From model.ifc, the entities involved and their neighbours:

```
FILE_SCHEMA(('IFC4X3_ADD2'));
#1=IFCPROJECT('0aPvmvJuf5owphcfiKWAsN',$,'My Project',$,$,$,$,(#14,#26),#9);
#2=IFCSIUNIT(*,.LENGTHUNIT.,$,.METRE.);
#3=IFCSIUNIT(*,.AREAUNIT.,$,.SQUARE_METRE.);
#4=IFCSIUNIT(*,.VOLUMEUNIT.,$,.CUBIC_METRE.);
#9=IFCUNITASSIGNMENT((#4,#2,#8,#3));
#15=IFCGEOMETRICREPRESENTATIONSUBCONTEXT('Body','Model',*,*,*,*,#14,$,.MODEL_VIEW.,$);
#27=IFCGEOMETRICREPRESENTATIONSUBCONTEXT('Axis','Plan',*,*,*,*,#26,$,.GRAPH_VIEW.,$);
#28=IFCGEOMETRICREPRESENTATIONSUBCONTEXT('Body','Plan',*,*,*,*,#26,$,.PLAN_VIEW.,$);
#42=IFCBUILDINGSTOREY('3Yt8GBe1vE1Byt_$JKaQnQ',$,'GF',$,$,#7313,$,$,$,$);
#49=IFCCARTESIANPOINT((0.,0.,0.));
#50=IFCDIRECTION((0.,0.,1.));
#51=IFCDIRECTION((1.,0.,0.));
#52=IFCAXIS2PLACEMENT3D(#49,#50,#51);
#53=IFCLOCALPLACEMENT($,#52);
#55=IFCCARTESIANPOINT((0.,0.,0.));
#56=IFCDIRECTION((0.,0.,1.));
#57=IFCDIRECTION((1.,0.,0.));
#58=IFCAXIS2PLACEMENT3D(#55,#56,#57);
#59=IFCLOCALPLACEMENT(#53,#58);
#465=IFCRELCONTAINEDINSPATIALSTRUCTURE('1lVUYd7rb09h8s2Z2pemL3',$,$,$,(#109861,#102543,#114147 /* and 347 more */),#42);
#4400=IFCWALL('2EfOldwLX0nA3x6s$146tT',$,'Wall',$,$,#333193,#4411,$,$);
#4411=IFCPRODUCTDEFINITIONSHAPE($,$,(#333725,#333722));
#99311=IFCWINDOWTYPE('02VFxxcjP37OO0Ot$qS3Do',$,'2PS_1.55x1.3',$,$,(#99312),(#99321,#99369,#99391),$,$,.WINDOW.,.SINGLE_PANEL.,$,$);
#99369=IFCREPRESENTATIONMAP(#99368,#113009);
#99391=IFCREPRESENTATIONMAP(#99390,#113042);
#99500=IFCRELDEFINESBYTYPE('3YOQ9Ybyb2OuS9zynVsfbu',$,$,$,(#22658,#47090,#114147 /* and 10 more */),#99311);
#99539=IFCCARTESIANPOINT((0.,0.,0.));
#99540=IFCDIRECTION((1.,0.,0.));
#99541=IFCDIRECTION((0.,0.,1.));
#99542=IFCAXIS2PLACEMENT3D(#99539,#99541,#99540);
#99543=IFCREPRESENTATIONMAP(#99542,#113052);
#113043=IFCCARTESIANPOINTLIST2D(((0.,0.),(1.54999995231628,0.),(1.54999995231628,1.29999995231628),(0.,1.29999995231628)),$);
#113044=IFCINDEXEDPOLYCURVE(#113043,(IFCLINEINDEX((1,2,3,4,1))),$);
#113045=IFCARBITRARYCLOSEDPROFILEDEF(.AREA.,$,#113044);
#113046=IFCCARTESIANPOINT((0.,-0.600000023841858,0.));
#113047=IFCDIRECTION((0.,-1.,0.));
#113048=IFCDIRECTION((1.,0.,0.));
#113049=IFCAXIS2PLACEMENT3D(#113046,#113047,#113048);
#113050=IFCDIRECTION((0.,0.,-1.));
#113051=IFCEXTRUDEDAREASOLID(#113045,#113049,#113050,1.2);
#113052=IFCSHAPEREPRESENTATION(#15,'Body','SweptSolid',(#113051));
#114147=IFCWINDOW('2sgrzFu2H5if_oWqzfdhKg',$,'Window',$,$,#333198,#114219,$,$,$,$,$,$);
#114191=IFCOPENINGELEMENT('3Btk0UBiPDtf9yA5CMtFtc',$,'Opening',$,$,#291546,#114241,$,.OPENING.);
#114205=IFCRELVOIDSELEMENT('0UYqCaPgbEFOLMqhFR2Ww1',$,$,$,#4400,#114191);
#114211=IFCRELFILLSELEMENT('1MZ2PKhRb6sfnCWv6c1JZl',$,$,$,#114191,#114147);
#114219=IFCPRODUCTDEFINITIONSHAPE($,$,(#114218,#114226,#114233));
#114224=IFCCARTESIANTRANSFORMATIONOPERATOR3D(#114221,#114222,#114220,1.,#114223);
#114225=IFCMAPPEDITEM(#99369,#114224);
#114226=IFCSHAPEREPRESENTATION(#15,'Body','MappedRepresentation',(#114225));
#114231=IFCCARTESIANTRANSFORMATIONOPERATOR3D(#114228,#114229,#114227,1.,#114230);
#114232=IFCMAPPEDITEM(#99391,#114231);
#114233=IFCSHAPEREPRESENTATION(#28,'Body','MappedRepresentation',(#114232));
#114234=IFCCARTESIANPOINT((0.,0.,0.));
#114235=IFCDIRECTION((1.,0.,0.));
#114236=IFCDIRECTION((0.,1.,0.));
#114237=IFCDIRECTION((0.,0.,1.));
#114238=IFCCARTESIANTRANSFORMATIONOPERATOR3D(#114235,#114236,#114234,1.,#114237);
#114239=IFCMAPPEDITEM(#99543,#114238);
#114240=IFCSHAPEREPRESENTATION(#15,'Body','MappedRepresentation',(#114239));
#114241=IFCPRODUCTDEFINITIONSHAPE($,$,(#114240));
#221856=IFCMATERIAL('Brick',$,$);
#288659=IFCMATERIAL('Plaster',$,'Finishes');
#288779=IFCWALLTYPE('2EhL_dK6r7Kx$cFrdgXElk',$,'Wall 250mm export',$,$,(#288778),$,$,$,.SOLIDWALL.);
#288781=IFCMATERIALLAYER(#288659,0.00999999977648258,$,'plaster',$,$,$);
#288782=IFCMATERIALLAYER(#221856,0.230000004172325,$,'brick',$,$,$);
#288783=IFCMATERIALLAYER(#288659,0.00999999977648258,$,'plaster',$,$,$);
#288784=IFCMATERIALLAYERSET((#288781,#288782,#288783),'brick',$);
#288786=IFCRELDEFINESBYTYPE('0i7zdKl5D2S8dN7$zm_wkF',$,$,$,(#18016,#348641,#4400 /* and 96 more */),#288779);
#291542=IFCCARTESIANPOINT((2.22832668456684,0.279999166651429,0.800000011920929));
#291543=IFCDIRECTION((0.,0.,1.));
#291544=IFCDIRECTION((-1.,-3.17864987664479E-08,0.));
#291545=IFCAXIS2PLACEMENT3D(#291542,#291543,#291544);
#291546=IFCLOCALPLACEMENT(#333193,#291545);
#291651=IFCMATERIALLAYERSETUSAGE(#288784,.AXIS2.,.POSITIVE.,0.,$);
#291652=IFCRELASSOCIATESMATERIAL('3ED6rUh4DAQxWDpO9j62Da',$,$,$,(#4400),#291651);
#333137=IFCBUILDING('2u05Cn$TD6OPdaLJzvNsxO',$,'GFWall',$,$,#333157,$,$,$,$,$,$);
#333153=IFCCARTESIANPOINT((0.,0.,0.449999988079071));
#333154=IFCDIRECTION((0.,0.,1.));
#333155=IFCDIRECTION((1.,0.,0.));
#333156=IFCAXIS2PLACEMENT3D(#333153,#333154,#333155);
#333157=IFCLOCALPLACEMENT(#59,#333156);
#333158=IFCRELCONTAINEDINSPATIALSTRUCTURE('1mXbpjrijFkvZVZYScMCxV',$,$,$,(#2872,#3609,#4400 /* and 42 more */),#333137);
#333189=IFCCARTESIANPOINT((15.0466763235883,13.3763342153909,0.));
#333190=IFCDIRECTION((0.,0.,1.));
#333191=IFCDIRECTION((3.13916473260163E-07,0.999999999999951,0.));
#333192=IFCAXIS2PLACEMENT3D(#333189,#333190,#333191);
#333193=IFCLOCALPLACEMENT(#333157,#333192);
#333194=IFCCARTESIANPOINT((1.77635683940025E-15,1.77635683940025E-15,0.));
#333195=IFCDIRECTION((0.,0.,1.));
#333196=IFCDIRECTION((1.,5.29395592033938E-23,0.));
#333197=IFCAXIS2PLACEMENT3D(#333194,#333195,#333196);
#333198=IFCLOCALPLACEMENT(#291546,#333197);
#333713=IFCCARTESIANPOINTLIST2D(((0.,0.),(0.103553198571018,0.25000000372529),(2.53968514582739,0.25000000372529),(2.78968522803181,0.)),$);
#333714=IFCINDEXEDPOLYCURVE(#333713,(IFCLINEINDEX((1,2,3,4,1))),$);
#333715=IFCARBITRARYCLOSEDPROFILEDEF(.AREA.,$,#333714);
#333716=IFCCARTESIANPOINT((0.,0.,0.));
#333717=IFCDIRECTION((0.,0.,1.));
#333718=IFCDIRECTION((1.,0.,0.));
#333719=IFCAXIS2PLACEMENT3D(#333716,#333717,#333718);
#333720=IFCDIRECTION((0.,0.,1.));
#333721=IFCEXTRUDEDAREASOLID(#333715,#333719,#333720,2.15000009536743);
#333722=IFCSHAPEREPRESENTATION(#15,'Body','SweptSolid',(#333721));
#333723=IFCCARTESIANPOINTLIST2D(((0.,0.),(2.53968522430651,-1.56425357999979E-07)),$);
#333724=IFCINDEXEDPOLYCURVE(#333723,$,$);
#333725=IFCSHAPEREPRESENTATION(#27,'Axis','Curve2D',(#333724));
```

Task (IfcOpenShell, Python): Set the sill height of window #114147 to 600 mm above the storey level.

```python
import numpy as np
import ifcopenshell
import ifcopenshell.api.geometry
import ifcopenshell.geom
import ifcopenshell.util.element
import ifcopenshell.util.placement
import ifcopenshell.util.shape
import ifcopenshell.util.unit

model = ifcopenshell.open("model.ifc")
unit_scale = ifcopenshell.util.unit.calculate_unit_scale(model)

window = model.by_guid("2sgrzFu2H5if_oWqzfdhKg")
opening = window.FillsVoids[0].RelatingOpeningElement
storey = ifcopenshell.util.element.get_container(window, ifc_class="IfcBuildingStorey")
level = ifcopenshell.util.placement.get_local_placement(storey.ObjectPlacement)[2, 3]

# The opening's origin need not be at the sill, so measure its lowest point.
shape = ifcopenshell.geom.create_shape(ifcopenshell.geom.settings(), opening)
bottom = ifcopenshell.util.shape.get_shape_bottom_elevation(shape, shape.geometry) / unit_scale
dz = level + 0.6 / unit_scale - bottom

shift = np.array([0.0, 0.0, dz])
# The window is placed relative to its opening, so it follows when the opening moves.
matrix = ifcopenshell.util.placement.get_local_placement(opening.ObjectPlacement)
matrix[:3, 3] += shift
ifcopenshell.api.geometry.edit_object_placement(
    model, product=opening, matrix=matrix, is_si=False, should_transform_children=True
)

print(f"moved by {dz * unit_scale:+.3f} m")

model.write("model_updated.ifc")
```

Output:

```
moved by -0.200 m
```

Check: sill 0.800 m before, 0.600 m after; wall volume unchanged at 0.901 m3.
